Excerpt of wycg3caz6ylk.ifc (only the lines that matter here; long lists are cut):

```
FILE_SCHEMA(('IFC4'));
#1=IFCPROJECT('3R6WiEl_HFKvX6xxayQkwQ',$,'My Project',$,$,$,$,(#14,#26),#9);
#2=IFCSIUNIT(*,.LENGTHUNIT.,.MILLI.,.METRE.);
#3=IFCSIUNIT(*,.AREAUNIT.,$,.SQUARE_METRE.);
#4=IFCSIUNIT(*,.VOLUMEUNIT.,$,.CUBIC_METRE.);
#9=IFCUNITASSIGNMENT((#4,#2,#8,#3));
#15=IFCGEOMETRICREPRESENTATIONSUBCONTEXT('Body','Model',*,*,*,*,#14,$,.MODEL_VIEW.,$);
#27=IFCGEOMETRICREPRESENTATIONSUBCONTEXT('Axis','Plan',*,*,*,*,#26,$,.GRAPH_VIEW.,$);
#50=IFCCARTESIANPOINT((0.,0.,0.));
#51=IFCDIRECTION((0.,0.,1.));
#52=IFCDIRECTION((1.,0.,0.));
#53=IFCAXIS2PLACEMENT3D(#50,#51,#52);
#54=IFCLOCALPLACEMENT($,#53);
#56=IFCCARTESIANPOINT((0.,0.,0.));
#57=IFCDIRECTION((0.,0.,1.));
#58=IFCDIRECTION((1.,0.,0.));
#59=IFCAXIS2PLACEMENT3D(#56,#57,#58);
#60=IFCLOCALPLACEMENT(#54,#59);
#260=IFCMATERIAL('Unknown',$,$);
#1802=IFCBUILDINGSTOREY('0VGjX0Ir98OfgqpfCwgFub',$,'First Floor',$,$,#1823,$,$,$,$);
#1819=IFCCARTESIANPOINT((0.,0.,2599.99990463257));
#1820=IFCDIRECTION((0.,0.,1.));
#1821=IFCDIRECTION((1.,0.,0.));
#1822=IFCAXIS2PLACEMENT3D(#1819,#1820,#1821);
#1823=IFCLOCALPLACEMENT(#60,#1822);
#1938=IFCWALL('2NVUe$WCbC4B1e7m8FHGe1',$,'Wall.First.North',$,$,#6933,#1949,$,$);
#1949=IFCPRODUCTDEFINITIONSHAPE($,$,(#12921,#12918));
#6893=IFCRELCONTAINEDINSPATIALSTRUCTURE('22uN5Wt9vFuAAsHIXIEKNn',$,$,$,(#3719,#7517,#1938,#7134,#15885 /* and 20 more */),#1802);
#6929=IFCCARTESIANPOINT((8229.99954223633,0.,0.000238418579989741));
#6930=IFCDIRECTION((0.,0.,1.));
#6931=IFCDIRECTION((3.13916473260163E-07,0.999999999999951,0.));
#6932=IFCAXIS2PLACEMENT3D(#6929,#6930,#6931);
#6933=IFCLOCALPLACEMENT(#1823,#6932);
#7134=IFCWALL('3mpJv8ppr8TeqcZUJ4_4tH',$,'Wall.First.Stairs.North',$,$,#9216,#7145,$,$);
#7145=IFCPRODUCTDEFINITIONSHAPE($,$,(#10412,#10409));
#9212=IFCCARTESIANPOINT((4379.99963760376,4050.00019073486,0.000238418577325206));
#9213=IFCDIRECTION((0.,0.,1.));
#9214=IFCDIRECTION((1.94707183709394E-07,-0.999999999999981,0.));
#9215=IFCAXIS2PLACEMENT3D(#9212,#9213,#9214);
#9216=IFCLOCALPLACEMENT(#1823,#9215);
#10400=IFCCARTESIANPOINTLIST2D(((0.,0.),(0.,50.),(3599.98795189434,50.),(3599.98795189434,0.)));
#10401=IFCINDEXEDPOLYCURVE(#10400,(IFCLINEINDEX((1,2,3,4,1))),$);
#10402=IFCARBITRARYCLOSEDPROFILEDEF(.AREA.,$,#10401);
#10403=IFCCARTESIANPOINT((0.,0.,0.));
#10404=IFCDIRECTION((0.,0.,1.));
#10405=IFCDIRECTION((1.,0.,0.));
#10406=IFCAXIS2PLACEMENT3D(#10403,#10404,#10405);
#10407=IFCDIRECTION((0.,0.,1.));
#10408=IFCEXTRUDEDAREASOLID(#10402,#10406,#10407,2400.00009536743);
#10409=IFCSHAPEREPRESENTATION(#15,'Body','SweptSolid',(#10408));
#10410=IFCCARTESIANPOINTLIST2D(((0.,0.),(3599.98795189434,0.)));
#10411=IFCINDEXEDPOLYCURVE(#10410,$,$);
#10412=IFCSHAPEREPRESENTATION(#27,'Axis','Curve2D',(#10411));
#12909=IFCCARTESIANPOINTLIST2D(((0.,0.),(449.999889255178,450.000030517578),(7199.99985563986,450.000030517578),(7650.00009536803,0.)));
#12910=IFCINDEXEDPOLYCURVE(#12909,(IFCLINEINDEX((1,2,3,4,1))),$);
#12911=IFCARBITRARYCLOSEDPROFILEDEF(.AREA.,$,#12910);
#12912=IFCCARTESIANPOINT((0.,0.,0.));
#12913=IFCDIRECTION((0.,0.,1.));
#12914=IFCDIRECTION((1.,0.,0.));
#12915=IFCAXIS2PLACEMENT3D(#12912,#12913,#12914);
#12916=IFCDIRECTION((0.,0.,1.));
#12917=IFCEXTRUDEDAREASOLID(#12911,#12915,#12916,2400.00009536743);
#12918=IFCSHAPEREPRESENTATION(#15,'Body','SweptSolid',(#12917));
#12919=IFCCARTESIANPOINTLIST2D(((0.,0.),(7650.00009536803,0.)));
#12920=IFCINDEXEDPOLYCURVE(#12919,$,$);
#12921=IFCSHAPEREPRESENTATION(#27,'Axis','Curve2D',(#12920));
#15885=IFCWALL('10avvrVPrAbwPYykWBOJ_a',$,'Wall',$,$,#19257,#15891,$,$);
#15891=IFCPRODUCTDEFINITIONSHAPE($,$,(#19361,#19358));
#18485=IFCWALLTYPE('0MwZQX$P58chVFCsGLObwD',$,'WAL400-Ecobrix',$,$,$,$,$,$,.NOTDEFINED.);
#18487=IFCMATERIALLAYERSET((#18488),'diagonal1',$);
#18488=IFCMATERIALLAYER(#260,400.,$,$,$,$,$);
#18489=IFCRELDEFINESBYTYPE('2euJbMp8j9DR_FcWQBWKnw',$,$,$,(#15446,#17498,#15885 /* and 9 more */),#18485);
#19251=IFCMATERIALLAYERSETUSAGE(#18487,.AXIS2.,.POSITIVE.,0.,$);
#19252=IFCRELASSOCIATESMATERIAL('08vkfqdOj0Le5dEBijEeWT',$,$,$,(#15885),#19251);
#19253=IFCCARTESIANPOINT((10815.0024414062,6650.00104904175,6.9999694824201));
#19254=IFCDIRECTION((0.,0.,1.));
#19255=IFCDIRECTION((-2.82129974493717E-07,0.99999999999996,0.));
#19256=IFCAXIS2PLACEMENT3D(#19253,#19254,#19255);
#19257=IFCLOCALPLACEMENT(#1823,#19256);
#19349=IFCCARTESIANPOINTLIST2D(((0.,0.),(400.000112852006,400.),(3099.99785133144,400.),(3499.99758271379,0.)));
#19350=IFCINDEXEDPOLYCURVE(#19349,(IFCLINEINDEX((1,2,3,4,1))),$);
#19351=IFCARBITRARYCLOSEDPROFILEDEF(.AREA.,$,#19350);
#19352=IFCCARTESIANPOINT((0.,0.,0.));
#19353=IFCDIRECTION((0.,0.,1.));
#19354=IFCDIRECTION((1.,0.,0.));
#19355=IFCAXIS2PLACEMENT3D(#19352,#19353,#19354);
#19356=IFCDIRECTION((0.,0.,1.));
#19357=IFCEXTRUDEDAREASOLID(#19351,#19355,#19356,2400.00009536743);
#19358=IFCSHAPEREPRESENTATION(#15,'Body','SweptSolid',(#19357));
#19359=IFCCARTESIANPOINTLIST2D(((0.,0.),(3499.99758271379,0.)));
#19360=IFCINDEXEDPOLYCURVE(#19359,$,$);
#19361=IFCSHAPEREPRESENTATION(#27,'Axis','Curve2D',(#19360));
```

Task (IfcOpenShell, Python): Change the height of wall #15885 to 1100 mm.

```python
import ifcopenshell
import ifcopenshell.geom
import ifcopenshell.util.representation
import ifcopenshell.util.shape
import ifcopenshell.util.unit

model = ifcopenshell.open("wycg3caz6ylk.ifc")
unit_scale = ifcopenshell.util.unit.calculate_unit_scale(model)
settings = ifcopenshell.geom.settings()


def volume(element):
    """Net volume in cubic metres, openings subtracted."""
    shape = ifcopenshell.geom.create_shape(settings, element)
    return ifcopenshell.util.shape.get_volume(shape.geometry)


wall = model.by_guid("10avvrVPrAbwPYykWBOJ_a")
before = volume(wall)

body = ifcopenshell.util.representation.get_representation(wall, "Model", "Body")
solid = body.Items[0]
old_height = solid.Depth
solid.Depth = 1.1 / unit_scale
after = volume(wall)

print(f"height {old_height:g} -> {solid.Depth:g}, volume {before:.3f} -> {after:.3f} m3")

model.write("wycg3caz6ylk_rev.ifc")
```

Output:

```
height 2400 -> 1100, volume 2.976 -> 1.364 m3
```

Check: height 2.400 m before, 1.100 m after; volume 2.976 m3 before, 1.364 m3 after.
